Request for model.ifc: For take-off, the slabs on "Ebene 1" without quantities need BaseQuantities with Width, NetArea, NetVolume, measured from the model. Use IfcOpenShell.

First a look at what the model holds.

```python
import ifcopenshell
import ifcopenshell.util.element
import ifcopenshell.util.unit

model = ifcopenshell.open("model.ifc")
print(model.schema)
for unit_type in ("LENGTHUNIT", "AREAUNIT", "VOLUMEUNIT"):
    print(unit_type, ifcopenshell.util.unit.calculate_unit_scale(model, unit_type))
storey = next(s for s in model.by_type("IfcBuildingStorey") if s.Name == "Ebene 1")
slabs = [e for e in ifcopenshell.util.element.get_decomposition(storey) if e.is_a("IfcSlab")]
for e in sorted(slabs, key=lambda e: e.id()):
    print(e.id(), e.is_a(), e.Name, list(ifcopenshell.util.element.get_psets(e, qtos_only=True)), sep=" | ")
```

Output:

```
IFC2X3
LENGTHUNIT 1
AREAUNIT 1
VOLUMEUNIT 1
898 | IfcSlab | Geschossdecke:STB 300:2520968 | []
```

```python
import ifcopenshell
import ifcopenshell.api.pset
import ifcopenshell.geom
import ifcopenshell.util.element
import ifcopenshell.util.shape
import ifcopenshell.util.unit

model = ifcopenshell.open("model.ifc")
unit_scale = ifcopenshell.util.unit.calculate_unit_scale(model)
area_scale = ifcopenshell.util.unit.calculate_unit_scale(model, "AREAUNIT")
volume_scale = ifcopenshell.util.unit.calculate_unit_scale(model, "VOLUMEUNIT")
settings = ifcopenshell.geom.settings()

storey = next(s for s in model.by_type("IfcBuildingStorey") if s.Name == "Ebene 1")
slabs = [e for e in ifcopenshell.util.element.get_decomposition(storey) if e.is_a("IfcSlab")]

for e in sorted(slabs, key=lambda e: e.id()):
    if ifcopenshell.util.element.get_psets(e, qtos_only=True, should_inherit=False):
        continue
    # Geometry comes back in metres, in the element's own axes.
    shape = ifcopenshell.geom.create_shape(settings, e)
    values = {
        "Width": ifcopenshell.util.shape.get_z(shape.geometry) / unit_scale,
        "NetArea": ifcopenshell.util.shape.get_footprint_area(shape.geometry) / area_scale,
        "NetVolume": ifcopenshell.util.shape.get_volume(shape.geometry) / volume_scale,
    }
    qto = ifcopenshell.api.pset.add_qto(model, product=e, name="BaseQuantities")
    ifcopenshell.api.pset.edit_qto(model, qto=qto, properties=values)
    print(e.id(), {k: round(v, 3) for k, v in values.items()})

model.write("model_edited.ifc")
```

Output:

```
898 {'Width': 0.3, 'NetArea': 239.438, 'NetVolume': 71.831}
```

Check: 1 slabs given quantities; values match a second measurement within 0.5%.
